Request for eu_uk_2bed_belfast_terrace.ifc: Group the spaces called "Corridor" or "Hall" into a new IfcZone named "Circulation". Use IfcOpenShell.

First a look at what the model holds.

```python
import ifcopenshell

model = ifcopenshell.open("eu_uk_2bed_belfast_terrace.ifc")
print(model.schema)
seen = {}
for space in model.by_type("IfcSpace"):
    seen[space.LongName] = seen.get(space.LongName, 0) + 1
for name, count in sorted(seen.items(), key=str):
    print(count, "x", name)
print("zones:", [z.Name for z in model.by_type("IfcZone")][:20])
```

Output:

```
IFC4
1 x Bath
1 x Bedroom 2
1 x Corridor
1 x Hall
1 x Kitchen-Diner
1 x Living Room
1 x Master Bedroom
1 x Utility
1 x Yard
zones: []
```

```python
import ifcopenshell
import ifcopenshell.api.group
import ifcopenshell.api.root

model = ifcopenshell.open("eu_uk_2bed_belfast_terrace.ifc")

names = {"Corridor", "Hall"}
spaces = [s for s in model.by_type("IfcSpace") if s.LongName in names]

zone = ifcopenshell.api.root.create_entity(model, ifc_class="IfcZone", name="Circulation")
ifcopenshell.api.group.assign_group(model, products=spaces, group=zone)
print(len(spaces), "spaces in", zone.Name)

model.write("eu_uk_2bed_belfast_terrace_v2.ifc")
```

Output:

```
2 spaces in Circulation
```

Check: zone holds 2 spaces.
